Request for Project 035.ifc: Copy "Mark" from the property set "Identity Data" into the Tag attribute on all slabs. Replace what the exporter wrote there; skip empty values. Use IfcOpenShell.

First a look at what the model holds.

```python
import ifcopenshell
import ifcopenshell.util.element

model = ifcopenshell.open("Project 035.ifc")
print(model.schema)
slabs = model.by_type("IfcSlab")
print(len(slabs), "slabs")
for e in slabs[:8]:
    source = ifcopenshell.util.element.get_pset(e, "Identity Data", "Mark")
    target = e.Tag
    print(e.id(), repr(source), repr(target), sep=" | ")
```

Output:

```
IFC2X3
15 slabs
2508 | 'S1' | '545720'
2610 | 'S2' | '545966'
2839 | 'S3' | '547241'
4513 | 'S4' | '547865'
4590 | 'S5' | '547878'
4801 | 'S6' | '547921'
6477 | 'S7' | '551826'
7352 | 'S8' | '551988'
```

```python
import ifcopenshell
import ifcopenshell.util.element

model = ifcopenshell.open("Project 035.ifc")

count = 0
for e in model.by_type("IfcSlab"):
    value = ifcopenshell.util.element.get_pset(e, "Identity Data", "Mark")
    current = e.Tag
    if not value or not value.strip() or current == value:
        continue
    e.Tag = value
    count += 1

print(count, "slabs updated")

model.write("Project 035_updated.ifc")
```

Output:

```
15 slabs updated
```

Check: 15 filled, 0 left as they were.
